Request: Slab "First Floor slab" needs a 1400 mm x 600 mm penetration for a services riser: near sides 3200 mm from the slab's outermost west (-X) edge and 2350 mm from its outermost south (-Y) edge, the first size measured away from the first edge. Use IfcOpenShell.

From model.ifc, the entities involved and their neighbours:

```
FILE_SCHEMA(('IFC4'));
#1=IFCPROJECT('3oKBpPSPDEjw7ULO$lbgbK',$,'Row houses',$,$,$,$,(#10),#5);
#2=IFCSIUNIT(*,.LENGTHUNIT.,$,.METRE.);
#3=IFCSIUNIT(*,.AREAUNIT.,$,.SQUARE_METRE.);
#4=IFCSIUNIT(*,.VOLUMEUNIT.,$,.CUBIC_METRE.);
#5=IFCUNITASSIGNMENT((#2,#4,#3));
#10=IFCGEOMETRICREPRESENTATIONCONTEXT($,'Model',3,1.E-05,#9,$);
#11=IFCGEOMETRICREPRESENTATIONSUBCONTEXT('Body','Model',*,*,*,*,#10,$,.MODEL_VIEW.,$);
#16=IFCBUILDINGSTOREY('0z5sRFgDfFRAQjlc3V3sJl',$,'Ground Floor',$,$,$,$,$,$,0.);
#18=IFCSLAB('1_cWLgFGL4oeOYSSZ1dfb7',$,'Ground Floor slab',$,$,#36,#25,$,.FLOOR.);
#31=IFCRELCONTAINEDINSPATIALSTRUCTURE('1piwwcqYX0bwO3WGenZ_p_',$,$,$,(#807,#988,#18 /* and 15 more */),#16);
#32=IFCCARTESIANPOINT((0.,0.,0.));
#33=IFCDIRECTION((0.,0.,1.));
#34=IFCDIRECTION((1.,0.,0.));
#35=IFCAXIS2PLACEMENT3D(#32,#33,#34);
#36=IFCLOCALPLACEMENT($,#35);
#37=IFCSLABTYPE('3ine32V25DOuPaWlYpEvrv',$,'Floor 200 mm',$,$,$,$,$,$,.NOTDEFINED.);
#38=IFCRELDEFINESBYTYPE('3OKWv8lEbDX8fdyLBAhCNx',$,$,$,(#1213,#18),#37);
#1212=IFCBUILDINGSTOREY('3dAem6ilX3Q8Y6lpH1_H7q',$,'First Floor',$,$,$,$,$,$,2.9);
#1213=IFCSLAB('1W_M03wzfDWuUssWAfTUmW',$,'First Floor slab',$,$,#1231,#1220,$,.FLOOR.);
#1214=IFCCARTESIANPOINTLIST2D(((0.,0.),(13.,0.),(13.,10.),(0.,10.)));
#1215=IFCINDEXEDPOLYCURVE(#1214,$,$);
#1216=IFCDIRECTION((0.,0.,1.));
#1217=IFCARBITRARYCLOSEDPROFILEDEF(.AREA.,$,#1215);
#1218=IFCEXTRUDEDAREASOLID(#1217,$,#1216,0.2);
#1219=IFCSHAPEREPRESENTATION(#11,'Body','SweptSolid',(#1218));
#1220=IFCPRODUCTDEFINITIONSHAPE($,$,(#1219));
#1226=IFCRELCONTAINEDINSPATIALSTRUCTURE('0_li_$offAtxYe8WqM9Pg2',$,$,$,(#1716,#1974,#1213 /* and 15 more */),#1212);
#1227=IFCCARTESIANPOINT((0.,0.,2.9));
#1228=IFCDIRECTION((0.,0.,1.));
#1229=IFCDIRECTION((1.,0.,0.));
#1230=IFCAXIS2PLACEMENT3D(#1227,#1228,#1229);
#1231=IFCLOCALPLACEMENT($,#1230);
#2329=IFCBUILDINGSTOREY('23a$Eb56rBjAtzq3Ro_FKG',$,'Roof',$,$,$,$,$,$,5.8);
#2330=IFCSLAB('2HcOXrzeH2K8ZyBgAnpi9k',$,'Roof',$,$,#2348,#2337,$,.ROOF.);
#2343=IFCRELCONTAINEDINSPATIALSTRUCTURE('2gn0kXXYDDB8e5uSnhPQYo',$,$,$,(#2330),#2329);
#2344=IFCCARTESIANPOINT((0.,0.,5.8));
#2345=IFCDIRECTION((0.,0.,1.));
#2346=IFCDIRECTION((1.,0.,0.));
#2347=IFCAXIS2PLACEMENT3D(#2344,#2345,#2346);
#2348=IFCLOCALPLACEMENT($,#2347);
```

```python
import numpy as np
import ifcopenshell
import ifcopenshell.api.feature
import ifcopenshell.api.geometry
import ifcopenshell.api.root
import ifcopenshell.geom
import ifcopenshell.util.placement
import ifcopenshell.util.representation
import ifcopenshell.util.shape
import ifcopenshell.util.unit

model = ifcopenshell.open("model.ifc")
unit_scale = ifcopenshell.util.unit.calculate_unit_scale(model)
settings = ifcopenshell.geom.settings()


def volume(element):
    """Net volume in cubic metres, openings subtracted."""
    shape = ifcopenshell.geom.create_shape(settings, element)
    return ifcopenshell.util.shape.get_volume(shape.geometry)


slab = model.by_guid("1W_M03wzfDWuUssWAfTUmW")
before = volume(slab)

# Extent in the slab's own axes, in metres. The edges named are its -X and -Y sides.
slab_shape = ifcopenshell.geom.create_shape(settings, slab)
vertices = ifcopenshell.util.shape.get_vertices(slab_shape.geometry)
x_min, y_min, bottom = vertices.min(axis=0)
top = vertices[:, 2].max()

opening = ifcopenshell.api.root.create_entity(model, ifc_class="IfcOpeningElement", name="Services riser opening", predefined_type="OPENING")
context = ifcopenshell.util.representation.get_context(model, "Model", "Body", "MODEL_VIEW")
width, depth = 1.4, 0.6
outline = [(0.0, 0.0), (width, 0.0), (width, depth), (0.0, depth), (0.0, 0.0)]
# Overshoot both faces by 50 mm so the cut is clean.
shape = ifcopenshell.api.geometry.add_slab_representation(
    model, context=context, depth=top - bottom + 0.1, polyline=outline
)
ifcopenshell.api.geometry.assign_representation(model, product=opening, representation=shape)

matrix = ifcopenshell.util.placement.get_local_placement(slab.ObjectPlacement)
matrix[:, 3] = matrix @ np.append(np.array([x_min + 3.2, y_min + 2.35, bottom - 0.05]) / unit_scale, 1.0)
ifcopenshell.api.geometry.edit_object_placement(model, product=opening, matrix=matrix, is_si=False)
ifcopenshell.api.feature.add_feature(model, feature=opening, element=slab)

after = volume(slab)

print(f"slab volume {before:.3f} -> {after:.3f} m3")

model.write("model_updated.ifc")
```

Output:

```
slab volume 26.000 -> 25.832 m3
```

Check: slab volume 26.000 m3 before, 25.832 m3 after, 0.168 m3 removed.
